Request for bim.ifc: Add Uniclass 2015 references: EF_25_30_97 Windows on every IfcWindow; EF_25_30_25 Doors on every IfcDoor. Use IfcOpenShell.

First a look at what the model holds.

```python
import ifcopenshell

model = ifcopenshell.open("bim.ifc")
print(model.schema)
print("classifications:", [c.Name for c in model.by_type("IfcClassification")])
for ifc_class in ("IfcDoor", "IfcRoof", "IfcStair", "IfcWall", "IfcWindow"):
    print(ifc_class, len(model.by_type(ifc_class)))
```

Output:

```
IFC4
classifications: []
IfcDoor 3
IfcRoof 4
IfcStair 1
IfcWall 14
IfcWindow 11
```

```python
import ifcopenshell
import ifcopenshell.api.classification

model = ifcopenshell.open("bim.ifc")

system = ifcopenshell.api.classification.add_classification(model, classification="Uniclass 2015")

codes = {
    "IfcWindow": ("EF_25_30_97", "Windows"),
    "IfcDoor": ("EF_25_30_25", "Doors"),
}
for ifc_class, (code, name) in codes.items():
    products = model.by_type(ifc_class)
    ifcopenshell.api.classification.add_reference(
        model, products=products, classification=system, identification=code, name=name
    )
    print(code, len(products))

model.write("bim_v2.ifc")
```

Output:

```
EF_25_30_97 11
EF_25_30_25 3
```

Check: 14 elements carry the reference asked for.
